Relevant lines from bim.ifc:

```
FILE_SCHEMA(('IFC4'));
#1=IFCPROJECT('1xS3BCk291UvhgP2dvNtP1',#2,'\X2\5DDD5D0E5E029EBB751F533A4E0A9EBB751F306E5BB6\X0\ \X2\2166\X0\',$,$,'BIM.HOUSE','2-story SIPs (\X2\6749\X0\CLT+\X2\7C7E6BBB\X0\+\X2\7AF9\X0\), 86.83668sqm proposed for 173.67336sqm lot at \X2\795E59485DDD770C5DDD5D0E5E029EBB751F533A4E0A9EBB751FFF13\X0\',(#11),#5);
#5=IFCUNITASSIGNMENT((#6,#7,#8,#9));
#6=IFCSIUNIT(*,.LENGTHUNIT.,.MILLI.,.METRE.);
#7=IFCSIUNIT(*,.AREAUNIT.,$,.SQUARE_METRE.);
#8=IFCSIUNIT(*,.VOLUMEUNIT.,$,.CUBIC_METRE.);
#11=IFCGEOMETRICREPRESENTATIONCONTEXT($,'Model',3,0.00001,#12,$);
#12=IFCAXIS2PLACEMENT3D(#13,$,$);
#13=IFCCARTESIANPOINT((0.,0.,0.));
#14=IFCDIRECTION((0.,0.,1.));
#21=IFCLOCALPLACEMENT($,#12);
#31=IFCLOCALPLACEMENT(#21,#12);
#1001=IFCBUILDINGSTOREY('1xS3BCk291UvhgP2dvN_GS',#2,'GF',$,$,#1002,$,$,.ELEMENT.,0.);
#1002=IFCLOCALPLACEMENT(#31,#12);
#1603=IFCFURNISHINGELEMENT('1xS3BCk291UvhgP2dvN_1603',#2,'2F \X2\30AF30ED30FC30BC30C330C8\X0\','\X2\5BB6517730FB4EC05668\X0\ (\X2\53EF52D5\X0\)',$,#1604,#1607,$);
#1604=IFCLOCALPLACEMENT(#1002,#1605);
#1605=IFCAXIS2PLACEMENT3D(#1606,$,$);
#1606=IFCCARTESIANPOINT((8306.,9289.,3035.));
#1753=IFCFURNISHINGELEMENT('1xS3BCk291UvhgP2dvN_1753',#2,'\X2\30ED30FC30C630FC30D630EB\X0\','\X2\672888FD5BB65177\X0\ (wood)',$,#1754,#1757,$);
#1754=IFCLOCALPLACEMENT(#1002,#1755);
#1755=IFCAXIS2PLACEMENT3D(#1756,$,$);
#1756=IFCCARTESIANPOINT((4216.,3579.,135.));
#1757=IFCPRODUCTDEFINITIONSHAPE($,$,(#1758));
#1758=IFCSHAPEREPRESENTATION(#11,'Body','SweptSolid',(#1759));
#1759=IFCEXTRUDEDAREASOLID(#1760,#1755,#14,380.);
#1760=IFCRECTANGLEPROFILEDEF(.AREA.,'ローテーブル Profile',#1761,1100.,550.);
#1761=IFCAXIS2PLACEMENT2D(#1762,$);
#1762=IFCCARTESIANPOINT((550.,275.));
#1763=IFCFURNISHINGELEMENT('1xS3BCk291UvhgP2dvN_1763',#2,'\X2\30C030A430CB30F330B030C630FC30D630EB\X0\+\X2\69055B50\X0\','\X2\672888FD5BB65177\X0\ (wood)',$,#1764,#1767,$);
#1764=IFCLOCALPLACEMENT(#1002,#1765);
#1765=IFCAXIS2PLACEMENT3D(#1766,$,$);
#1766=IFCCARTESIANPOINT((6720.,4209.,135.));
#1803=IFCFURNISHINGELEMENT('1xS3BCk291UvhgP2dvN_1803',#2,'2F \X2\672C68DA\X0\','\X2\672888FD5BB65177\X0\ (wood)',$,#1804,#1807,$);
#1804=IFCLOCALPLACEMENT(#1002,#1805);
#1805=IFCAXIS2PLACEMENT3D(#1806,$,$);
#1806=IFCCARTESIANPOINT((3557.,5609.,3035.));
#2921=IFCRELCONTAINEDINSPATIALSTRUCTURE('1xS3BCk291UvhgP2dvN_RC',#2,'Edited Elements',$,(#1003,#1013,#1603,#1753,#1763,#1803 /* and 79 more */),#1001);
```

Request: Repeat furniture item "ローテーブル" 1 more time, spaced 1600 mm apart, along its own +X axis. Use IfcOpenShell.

```python
import ifcopenshell
import ifcopenshell.api.geometry
import ifcopenshell.api.root
import ifcopenshell.util.element
import ifcopenshell.util.placement
import ifcopenshell.util.unit

model = ifcopenshell.open("bim.ifc")
unit_scale = ifcopenshell.util.unit.calculate_unit_scale(model)


def reuse_history(source, copy):
    """copy_class also copies each property set's owner history, people and application; keep the originals."""
    for rel in copy.IsDefinedBy:
        if rel.is_a("IfcRelDefinesByProperties") and (history := rel.RelatingPropertyDefinition.OwnerHistory):
            rel.RelatingPropertyDefinition.OwnerHistory = source.OwnerHistory
            ifcopenshell.util.element.remove_deep2(model, history)


source = model.by_id(1753)
base = ifcopenshell.util.placement.get_local_placement(source.ObjectPlacement)
step = base[:3, 0] * 1.6 / unit_scale

for i in range(1, 2):
    copy = ifcopenshell.api.root.copy_class(model, product=source)
    copy.Representation = ifcopenshell.util.element.copy_deep(
        model, source.Representation, exclude=["IfcGeometricRepresentationContext", "IfcRepresentationMap"]
    )
    reuse_history(source, copy)
    matrix = base.copy()
    matrix[:3, 3] += i * step
    print("added at", matrix[:3, 3].round(3) + 0.0)
    ifcopenshell.api.geometry.edit_object_placement(model, product=copy, matrix=matrix, is_si=False)

model.write("bim_updated.ifc")
```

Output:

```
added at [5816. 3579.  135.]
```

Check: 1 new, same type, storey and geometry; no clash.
